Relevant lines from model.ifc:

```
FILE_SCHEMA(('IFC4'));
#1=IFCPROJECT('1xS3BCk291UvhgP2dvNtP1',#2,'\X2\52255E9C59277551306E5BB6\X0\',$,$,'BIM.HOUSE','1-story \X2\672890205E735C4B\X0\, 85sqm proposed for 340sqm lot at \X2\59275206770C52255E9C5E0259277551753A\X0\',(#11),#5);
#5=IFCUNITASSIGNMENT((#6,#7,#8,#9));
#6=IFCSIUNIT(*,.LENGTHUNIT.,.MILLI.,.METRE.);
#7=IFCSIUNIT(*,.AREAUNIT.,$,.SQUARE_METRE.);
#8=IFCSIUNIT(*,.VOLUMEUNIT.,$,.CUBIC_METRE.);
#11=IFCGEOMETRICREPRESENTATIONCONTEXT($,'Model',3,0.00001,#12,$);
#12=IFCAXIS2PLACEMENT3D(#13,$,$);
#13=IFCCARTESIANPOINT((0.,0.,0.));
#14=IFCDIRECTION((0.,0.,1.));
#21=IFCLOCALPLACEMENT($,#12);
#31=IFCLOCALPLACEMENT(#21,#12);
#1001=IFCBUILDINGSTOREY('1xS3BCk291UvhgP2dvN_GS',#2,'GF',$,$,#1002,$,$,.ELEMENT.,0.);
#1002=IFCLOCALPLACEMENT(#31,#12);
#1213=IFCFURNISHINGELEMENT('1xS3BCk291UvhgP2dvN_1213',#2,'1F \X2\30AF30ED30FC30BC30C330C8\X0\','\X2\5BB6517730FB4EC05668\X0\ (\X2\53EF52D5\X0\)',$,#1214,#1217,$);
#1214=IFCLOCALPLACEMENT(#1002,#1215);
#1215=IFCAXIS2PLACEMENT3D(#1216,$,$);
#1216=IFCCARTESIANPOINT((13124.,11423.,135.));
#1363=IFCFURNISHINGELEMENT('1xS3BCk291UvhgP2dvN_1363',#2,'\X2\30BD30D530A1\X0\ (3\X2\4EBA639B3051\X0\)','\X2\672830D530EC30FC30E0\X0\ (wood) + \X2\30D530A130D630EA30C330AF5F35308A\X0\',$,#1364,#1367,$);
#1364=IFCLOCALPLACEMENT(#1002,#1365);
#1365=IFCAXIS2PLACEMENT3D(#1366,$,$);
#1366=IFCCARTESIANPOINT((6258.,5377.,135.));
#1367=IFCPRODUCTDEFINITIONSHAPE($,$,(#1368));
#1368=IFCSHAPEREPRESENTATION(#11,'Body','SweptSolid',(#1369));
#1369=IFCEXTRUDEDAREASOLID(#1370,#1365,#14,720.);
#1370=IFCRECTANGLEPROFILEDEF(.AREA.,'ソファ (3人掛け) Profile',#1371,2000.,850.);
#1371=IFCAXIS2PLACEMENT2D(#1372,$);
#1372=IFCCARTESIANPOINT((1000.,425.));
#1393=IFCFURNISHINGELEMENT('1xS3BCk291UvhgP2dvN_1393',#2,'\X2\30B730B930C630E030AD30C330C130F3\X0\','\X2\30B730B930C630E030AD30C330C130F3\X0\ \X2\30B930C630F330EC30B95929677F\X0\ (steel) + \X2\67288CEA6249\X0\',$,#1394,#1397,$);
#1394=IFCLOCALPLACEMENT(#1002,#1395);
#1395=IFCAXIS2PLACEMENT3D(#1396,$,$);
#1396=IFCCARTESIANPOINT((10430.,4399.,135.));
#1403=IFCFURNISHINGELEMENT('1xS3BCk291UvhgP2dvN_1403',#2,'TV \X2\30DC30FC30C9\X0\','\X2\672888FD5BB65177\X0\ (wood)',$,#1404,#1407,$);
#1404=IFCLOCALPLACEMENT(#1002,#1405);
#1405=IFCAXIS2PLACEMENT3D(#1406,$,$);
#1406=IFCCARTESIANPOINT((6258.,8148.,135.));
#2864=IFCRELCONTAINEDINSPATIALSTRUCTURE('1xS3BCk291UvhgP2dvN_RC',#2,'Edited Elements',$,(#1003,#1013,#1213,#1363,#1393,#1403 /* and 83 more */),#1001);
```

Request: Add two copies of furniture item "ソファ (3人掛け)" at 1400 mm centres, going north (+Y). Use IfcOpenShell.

```python
import numpy as np
import ifcopenshell
import ifcopenshell.api.geometry
import ifcopenshell.api.root
import ifcopenshell.util.element
import ifcopenshell.util.placement
import ifcopenshell.util.unit

model = ifcopenshell.open("model.ifc")
unit_scale = ifcopenshell.util.unit.calculate_unit_scale(model)


def reuse_history(source, copy):
    """copy_class also copies each property set's owner history, people and application; keep the originals."""
    for rel in copy.IsDefinedBy:
        if rel.is_a("IfcRelDefinesByProperties") and (history := rel.RelatingPropertyDefinition.OwnerHistory):
            rel.RelatingPropertyDefinition.OwnerHistory = source.OwnerHistory
            ifcopenshell.util.element.remove_deep2(model, history)


source = model.by_id(1363)
base = ifcopenshell.util.placement.get_local_placement(source.ObjectPlacement)
step = np.array([0.0, 1.0, 0.0]) * 1.4 / unit_scale

for i in range(1, 3):
    copy = ifcopenshell.api.root.copy_class(model, product=source)
    copy.Representation = ifcopenshell.util.element.copy_deep(
        model, source.Representation, exclude=["IfcGeometricRepresentationContext", "IfcRepresentationMap"]
    )
    reuse_history(source, copy)
    matrix = base.copy()
    matrix[:3, 3] += i * step
    print("added at", matrix[:3, 3].round(3) + 0.0)
    ifcopenshell.api.geometry.edit_object_placement(model, product=copy, matrix=matrix, is_si=False)

model.write("model-out.ifc")
```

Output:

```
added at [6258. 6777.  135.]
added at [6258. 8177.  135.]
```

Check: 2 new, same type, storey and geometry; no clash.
